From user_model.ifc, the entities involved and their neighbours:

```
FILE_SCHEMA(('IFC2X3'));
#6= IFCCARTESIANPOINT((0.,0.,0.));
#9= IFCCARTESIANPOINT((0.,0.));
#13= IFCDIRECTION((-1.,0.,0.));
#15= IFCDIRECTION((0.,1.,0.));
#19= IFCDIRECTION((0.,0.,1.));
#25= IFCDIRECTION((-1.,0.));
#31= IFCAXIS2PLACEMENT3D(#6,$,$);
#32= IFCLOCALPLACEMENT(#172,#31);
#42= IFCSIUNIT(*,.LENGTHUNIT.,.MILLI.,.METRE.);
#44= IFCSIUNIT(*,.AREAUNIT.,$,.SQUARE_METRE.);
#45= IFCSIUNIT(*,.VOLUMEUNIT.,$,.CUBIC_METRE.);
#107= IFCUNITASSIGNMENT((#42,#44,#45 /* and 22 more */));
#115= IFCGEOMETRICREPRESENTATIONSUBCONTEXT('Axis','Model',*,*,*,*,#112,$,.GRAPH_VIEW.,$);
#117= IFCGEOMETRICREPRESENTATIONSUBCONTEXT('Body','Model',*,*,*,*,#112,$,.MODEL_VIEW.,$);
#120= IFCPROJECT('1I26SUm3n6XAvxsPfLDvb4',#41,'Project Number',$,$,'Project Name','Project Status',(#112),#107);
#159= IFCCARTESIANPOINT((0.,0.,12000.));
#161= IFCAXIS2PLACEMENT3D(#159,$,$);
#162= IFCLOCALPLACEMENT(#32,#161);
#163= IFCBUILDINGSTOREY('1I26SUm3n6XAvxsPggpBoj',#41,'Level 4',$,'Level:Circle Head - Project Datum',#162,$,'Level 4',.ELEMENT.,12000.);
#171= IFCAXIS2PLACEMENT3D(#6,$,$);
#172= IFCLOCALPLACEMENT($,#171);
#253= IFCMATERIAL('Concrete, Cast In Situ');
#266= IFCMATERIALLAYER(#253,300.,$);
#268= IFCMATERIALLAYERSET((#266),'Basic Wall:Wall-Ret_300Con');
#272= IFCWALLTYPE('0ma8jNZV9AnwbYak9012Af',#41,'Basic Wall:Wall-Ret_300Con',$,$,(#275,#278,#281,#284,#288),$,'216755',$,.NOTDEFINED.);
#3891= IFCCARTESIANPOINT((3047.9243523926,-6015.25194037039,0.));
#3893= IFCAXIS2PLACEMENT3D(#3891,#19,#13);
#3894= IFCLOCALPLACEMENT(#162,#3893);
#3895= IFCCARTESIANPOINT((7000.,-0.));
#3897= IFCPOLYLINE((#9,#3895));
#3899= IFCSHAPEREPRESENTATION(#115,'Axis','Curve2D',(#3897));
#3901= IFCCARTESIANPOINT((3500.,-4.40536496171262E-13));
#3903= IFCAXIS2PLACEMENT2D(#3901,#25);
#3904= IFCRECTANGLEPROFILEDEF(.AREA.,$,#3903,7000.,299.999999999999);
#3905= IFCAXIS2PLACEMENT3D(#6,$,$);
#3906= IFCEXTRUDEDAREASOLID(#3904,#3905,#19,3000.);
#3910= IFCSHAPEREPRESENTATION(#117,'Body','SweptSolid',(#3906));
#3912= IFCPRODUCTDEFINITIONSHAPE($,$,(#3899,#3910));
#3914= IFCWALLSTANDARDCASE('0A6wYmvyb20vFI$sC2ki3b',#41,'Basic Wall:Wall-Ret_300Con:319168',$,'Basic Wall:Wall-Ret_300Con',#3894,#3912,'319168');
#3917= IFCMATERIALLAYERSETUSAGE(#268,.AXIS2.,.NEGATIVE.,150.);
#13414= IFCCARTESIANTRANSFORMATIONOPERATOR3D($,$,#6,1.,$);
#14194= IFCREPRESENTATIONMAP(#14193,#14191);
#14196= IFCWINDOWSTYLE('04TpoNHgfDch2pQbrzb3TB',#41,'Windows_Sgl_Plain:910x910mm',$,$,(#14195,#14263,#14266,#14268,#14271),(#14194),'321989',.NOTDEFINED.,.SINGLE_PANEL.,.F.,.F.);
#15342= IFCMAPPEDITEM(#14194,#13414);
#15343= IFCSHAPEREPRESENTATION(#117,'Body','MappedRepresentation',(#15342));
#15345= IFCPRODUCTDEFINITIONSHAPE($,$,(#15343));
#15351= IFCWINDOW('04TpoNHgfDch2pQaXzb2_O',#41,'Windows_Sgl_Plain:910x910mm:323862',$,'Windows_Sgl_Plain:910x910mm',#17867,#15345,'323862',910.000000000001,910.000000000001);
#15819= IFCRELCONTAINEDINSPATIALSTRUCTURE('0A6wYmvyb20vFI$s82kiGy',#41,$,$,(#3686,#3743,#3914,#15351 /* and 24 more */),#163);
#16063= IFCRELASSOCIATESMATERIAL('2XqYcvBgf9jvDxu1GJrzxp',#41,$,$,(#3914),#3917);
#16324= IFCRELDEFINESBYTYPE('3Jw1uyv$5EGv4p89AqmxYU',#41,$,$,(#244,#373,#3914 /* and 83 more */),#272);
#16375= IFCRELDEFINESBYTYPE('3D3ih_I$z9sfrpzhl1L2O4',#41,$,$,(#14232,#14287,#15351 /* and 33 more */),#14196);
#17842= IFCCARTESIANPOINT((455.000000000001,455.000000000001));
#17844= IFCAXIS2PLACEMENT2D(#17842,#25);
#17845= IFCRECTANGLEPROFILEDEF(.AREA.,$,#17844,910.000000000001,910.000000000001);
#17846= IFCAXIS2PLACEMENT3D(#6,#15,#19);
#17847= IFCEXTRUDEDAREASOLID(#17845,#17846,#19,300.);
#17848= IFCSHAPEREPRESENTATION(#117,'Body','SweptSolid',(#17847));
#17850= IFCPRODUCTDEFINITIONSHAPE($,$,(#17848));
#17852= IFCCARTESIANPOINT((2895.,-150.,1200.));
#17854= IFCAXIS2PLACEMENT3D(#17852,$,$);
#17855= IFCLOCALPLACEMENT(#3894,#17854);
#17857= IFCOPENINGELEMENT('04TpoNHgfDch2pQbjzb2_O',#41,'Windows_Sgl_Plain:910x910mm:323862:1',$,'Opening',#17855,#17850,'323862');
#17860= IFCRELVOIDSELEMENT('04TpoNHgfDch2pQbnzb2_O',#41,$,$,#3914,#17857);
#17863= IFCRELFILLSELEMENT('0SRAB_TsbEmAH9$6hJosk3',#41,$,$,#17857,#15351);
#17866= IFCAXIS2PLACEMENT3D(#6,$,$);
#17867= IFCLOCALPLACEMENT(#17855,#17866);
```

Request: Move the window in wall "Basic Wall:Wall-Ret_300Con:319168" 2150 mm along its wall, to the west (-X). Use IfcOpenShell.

```python
import ifcopenshell
import ifcopenshell.api.geometry
import ifcopenshell.util.placement

model = ifcopenshell.open("user_model.ifc")

window = model.by_guid("04TpoNHgfDch2pQaXzb2_O")
opening = window.FillsVoids[0].RelatingOpeningElement
wall = opening.VoidsElements[0].RelatingBuildingElement

wall_matrix = ifcopenshell.util.placement.get_local_placement(wall.ObjectPlacement)
shift = wall_matrix[:3, 0] * 2150.0
before = ifcopenshell.util.placement.get_local_placement(window.ObjectPlacement)[:3, 3].copy()

# The window is placed relative to its opening, so it follows when the opening moves.
matrix = ifcopenshell.util.placement.get_local_placement(opening.ObjectPlacement)
matrix[:3, 3] += shift
ifcopenshell.api.geometry.edit_object_placement(
    model, product=opening, matrix=matrix, is_si=False, should_transform_children=True
)

after = ifcopenshell.util.placement.get_local_placement(window.ObjectPlacement)[:3, 3]
print("window moved by", (after - before).round(3) + 0.0)

model.write("user_model_rev.ifc")
```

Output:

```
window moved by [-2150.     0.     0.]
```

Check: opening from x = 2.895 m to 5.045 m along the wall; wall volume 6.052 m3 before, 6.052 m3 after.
